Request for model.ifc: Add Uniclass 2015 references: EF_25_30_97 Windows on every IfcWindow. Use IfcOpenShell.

First a look at what the model holds.

```python
import ifcopenshell

model = ifcopenshell.open("model.ifc")
print(model.schema)
print("classifications:", [c.Name for c in model.by_type("IfcClassification")])
for ifc_class in ("IfcDoor", "IfcRoof", "IfcStair", "IfcWall", "IfcWindow"):
    print(ifc_class, len(model.by_type(ifc_class)))
```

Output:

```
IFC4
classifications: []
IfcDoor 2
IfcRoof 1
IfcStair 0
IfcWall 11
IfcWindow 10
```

```python
import ifcopenshell
import ifcopenshell.api.classification

model = ifcopenshell.open("model.ifc")

system = ifcopenshell.api.classification.add_classification(model, classification="Uniclass 2015")

codes = {
    "IfcWindow": ("EF_25_30_97", "Windows"),
}
for ifc_class, (code, name) in codes.items():
    products = model.by_type(ifc_class)
    ifcopenshell.api.classification.add_reference(
        model, products=products, classification=system, identification=code, name=name
    )
    print(code, len(products))

model.write("model_rev.ifc")
```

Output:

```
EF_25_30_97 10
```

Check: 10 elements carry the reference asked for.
